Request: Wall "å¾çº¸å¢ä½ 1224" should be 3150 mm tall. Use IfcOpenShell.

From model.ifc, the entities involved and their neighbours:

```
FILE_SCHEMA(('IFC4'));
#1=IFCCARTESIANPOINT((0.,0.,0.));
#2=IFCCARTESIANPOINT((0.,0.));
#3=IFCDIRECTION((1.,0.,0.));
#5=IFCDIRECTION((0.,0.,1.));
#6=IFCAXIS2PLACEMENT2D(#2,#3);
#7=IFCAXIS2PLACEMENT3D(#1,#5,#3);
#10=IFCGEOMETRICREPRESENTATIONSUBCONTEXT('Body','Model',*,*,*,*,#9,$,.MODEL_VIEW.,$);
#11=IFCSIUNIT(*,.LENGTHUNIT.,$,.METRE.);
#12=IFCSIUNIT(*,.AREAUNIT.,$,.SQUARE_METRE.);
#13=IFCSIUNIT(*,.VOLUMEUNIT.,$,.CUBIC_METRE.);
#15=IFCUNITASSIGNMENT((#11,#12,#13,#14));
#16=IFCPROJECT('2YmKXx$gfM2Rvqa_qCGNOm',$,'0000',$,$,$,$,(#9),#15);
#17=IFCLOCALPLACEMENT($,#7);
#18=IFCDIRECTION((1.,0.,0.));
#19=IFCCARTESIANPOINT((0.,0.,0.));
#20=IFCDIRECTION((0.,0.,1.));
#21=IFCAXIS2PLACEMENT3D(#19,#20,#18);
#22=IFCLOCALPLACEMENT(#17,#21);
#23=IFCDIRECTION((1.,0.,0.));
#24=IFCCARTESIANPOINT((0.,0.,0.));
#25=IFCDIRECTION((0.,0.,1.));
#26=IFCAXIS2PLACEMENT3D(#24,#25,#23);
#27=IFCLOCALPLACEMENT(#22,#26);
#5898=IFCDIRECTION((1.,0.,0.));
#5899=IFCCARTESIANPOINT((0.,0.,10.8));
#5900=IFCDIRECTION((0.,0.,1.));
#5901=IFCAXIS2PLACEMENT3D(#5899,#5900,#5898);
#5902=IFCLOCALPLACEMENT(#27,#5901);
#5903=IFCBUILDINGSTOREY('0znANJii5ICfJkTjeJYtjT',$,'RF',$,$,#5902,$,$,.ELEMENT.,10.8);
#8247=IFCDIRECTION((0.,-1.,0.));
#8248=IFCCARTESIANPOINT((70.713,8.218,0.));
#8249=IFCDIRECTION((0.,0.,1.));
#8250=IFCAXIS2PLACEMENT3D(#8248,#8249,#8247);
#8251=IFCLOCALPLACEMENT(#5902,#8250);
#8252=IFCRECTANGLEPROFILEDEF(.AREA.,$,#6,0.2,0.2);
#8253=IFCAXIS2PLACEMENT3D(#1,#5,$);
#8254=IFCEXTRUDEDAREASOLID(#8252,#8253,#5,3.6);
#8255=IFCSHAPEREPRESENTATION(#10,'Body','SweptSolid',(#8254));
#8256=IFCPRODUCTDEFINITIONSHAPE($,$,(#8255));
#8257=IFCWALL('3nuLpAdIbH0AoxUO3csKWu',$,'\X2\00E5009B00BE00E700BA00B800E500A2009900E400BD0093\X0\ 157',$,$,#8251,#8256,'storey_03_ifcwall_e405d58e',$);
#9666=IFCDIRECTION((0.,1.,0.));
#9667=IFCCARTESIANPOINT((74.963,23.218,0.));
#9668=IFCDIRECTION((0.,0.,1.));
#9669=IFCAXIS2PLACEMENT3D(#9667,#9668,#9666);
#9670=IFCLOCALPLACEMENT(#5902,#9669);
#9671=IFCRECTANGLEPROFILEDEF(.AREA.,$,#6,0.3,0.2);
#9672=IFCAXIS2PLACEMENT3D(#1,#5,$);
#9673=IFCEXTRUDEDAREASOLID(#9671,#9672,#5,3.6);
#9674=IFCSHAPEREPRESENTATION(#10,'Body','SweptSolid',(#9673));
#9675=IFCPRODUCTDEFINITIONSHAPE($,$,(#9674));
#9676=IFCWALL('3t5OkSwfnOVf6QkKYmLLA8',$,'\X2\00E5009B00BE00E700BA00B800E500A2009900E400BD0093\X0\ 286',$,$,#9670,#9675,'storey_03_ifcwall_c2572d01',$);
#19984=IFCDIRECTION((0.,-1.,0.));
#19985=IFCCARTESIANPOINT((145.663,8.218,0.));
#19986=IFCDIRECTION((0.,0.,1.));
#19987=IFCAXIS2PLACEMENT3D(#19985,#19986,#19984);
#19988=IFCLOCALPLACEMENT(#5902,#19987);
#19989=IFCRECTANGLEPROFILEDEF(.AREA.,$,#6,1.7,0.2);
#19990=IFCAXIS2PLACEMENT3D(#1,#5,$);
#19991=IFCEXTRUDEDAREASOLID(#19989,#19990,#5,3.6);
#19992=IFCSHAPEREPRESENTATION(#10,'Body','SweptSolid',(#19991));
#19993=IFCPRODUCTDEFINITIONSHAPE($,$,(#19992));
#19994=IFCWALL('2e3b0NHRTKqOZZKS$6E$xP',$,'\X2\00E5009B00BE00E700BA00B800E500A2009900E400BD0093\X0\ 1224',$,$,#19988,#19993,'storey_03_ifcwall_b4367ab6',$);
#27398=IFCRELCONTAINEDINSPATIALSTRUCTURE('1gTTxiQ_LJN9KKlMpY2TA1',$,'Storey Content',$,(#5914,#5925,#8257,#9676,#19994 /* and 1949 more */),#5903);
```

```python
import ifcopenshell
import ifcopenshell.geom
import ifcopenshell.util.representation
import ifcopenshell.util.shape

model = ifcopenshell.open("model.ifc")
settings = ifcopenshell.geom.settings()


def volume(element):
    """Net volume in cubic metres, openings subtracted."""
    shape = ifcopenshell.geom.create_shape(settings, element)
    return ifcopenshell.util.shape.get_volume(shape.geometry)


wall = model.by_id(19994)
before = volume(wall)

body = ifcopenshell.util.representation.get_representation(wall, "Model", "Body")
solid = body.Items[0]
old_height = solid.Depth
solid.Depth = 3.15
after = volume(wall)

print(f"height {old_height:g} -> {solid.Depth:g}, volume {before:.3f} -> {after:.3f} m3")

model.write("model_updated.ifc")
```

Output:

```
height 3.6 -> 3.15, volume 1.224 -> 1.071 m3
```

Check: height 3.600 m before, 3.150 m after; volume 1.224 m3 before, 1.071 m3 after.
